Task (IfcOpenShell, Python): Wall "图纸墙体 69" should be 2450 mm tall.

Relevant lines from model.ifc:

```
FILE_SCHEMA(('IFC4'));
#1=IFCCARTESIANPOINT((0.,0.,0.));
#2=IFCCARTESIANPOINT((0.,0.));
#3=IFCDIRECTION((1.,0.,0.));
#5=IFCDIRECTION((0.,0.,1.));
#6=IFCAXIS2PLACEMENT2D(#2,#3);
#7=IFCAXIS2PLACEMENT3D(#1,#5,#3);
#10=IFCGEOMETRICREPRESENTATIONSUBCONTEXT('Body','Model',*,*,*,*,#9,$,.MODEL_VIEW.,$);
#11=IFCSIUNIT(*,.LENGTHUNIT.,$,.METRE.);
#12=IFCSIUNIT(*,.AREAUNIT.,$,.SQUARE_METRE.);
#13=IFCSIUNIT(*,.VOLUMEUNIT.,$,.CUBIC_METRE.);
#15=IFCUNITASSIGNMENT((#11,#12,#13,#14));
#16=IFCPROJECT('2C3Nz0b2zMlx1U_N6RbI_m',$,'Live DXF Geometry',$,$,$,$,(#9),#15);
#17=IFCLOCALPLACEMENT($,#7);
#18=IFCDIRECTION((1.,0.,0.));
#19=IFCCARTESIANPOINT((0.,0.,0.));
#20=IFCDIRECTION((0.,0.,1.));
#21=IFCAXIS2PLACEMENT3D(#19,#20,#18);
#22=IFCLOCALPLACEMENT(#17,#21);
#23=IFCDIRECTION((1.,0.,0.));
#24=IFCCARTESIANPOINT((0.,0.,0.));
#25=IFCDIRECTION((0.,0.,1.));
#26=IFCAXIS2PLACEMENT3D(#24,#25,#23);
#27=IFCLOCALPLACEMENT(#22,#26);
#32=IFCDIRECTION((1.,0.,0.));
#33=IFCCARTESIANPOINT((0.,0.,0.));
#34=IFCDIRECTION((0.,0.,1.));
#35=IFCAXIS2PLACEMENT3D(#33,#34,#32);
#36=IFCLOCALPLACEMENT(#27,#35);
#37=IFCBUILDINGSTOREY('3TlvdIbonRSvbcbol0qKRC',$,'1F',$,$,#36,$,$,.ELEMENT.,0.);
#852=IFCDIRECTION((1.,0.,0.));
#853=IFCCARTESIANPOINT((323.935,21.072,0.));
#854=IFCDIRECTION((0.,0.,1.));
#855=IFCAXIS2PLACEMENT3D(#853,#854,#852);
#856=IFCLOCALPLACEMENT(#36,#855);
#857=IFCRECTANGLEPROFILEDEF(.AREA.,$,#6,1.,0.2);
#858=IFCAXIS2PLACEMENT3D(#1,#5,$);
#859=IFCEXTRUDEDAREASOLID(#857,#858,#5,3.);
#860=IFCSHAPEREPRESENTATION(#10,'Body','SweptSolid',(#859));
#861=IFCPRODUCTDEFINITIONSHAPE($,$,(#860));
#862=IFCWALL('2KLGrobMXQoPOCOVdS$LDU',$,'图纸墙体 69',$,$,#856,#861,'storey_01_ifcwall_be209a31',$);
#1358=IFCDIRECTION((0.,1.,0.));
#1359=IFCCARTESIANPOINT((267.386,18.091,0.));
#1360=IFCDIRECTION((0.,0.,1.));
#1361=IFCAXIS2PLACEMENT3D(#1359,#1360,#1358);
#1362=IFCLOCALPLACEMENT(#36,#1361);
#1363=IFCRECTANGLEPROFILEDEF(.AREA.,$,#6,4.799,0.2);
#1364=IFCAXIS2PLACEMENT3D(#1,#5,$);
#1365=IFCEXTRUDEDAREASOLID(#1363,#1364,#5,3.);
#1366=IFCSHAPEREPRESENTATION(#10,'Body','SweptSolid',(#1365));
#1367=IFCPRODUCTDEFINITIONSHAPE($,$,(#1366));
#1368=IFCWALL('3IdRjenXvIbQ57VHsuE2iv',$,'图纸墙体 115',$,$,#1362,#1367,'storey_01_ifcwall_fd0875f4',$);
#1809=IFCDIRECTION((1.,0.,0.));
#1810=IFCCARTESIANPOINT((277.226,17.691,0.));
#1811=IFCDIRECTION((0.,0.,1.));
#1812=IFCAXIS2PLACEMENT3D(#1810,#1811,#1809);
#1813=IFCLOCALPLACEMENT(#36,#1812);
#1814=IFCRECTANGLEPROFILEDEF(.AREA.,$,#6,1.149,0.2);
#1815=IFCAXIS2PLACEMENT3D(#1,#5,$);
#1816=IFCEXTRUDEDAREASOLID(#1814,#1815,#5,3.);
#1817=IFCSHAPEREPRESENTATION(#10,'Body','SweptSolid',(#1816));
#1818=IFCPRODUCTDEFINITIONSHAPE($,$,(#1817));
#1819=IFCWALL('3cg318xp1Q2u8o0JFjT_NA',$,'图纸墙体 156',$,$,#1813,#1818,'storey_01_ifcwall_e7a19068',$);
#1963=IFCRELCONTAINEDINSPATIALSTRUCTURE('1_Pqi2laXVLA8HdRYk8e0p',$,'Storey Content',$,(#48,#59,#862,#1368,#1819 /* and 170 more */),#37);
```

```python
import ifcopenshell
import ifcopenshell.geom
import ifcopenshell.util.representation
import ifcopenshell.util.shape
import ifcopenshell.util.unit

model = ifcopenshell.open("model.ifc")
unit_scale = ifcopenshell.util.unit.calculate_unit_scale(model)
settings = ifcopenshell.geom.settings()


def volume(element):
    """Net volume in cubic metres, openings subtracted."""
    shape = ifcopenshell.geom.create_shape(settings, element)
    return ifcopenshell.util.shape.get_volume(shape.geometry)


wall = model.by_guid("2KLGrobMXQoPOCOVdS$LDU")
before = volume(wall)

body = ifcopenshell.util.representation.get_representation(wall, "Model", "Body")
solid = body.Items[0]
old_height = solid.Depth
solid.Depth = 2.45 / unit_scale
after = volume(wall)

print(f"height {old_height:g} -> {solid.Depth:g}, volume {before:.3f} -> {after:.3f} m3")

model.write("model_rev.ifc")
```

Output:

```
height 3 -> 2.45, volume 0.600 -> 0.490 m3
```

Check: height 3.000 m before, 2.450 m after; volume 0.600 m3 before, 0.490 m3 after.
